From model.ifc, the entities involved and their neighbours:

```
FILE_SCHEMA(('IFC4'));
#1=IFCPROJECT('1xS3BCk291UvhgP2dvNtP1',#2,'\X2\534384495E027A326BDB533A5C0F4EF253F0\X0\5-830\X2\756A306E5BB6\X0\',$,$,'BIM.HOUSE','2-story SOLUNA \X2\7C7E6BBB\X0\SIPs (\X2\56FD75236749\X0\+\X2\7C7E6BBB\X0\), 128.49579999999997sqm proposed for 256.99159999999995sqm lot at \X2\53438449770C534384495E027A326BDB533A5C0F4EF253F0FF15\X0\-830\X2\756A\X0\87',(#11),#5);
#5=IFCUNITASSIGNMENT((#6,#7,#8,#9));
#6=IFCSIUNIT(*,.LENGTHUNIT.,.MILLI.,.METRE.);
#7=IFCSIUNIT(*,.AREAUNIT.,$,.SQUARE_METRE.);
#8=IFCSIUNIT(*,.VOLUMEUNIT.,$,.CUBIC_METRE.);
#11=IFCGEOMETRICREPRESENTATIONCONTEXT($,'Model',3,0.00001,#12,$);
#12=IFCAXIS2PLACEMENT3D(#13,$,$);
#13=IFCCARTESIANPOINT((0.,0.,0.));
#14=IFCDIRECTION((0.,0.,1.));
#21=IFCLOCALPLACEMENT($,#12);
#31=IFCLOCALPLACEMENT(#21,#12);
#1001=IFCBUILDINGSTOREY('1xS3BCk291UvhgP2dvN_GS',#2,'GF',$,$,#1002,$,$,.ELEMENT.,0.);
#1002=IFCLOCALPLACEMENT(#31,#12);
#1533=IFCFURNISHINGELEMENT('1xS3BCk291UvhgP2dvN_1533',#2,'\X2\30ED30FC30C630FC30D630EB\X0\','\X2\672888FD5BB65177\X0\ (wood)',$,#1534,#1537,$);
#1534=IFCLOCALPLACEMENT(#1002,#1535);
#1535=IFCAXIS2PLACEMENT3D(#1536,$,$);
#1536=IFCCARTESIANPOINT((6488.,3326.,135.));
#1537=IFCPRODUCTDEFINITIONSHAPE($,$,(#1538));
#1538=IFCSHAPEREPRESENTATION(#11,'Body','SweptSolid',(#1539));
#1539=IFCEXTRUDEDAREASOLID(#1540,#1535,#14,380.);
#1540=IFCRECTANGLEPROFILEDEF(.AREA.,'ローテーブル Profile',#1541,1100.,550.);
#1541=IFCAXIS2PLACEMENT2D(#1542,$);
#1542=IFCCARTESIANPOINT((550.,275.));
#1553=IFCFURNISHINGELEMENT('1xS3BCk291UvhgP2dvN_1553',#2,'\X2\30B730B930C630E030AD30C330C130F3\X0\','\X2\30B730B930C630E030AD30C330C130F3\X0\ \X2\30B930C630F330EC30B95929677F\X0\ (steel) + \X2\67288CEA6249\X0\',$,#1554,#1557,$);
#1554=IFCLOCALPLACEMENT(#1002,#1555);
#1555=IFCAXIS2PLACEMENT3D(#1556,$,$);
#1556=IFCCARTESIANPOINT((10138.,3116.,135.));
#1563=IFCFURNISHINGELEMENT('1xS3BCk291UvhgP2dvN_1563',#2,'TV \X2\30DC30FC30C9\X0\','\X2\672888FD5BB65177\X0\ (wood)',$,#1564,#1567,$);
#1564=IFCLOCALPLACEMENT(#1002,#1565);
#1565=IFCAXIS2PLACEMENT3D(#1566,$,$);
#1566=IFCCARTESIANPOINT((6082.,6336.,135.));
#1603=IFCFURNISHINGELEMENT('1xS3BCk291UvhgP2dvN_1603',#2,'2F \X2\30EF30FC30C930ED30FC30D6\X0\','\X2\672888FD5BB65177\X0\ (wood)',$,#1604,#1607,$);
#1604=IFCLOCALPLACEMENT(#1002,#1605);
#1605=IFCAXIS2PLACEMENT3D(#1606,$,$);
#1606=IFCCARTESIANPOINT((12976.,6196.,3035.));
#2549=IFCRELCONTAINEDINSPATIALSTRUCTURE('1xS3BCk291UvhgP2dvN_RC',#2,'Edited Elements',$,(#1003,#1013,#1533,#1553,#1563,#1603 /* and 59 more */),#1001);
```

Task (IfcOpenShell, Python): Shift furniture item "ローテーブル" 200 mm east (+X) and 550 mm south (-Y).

```python
import ifcopenshell
import ifcopenshell.api.geometry
import ifcopenshell.util.placement

model = ifcopenshell.open("model.ifc")

item = model.by_guid("1xS3BCk291UvhgP2dvN_1533")
matrix = ifcopenshell.util.placement.get_local_placement(item.ObjectPlacement)
matrix[0, 3] += 200.0
matrix[1, 3] -= 550.0
ifcopenshell.api.geometry.edit_object_placement(model, product=item, matrix=matrix, is_si=False)

print(ifcopenshell.util.placement.get_local_placement(item.ObjectPlacement).round(3) + 0.0)

model.write("model_updated.ifc")
```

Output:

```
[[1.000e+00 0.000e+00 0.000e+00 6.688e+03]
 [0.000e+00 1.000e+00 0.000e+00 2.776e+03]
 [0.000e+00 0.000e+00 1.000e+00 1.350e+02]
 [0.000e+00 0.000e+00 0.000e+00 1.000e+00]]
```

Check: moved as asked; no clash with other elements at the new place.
